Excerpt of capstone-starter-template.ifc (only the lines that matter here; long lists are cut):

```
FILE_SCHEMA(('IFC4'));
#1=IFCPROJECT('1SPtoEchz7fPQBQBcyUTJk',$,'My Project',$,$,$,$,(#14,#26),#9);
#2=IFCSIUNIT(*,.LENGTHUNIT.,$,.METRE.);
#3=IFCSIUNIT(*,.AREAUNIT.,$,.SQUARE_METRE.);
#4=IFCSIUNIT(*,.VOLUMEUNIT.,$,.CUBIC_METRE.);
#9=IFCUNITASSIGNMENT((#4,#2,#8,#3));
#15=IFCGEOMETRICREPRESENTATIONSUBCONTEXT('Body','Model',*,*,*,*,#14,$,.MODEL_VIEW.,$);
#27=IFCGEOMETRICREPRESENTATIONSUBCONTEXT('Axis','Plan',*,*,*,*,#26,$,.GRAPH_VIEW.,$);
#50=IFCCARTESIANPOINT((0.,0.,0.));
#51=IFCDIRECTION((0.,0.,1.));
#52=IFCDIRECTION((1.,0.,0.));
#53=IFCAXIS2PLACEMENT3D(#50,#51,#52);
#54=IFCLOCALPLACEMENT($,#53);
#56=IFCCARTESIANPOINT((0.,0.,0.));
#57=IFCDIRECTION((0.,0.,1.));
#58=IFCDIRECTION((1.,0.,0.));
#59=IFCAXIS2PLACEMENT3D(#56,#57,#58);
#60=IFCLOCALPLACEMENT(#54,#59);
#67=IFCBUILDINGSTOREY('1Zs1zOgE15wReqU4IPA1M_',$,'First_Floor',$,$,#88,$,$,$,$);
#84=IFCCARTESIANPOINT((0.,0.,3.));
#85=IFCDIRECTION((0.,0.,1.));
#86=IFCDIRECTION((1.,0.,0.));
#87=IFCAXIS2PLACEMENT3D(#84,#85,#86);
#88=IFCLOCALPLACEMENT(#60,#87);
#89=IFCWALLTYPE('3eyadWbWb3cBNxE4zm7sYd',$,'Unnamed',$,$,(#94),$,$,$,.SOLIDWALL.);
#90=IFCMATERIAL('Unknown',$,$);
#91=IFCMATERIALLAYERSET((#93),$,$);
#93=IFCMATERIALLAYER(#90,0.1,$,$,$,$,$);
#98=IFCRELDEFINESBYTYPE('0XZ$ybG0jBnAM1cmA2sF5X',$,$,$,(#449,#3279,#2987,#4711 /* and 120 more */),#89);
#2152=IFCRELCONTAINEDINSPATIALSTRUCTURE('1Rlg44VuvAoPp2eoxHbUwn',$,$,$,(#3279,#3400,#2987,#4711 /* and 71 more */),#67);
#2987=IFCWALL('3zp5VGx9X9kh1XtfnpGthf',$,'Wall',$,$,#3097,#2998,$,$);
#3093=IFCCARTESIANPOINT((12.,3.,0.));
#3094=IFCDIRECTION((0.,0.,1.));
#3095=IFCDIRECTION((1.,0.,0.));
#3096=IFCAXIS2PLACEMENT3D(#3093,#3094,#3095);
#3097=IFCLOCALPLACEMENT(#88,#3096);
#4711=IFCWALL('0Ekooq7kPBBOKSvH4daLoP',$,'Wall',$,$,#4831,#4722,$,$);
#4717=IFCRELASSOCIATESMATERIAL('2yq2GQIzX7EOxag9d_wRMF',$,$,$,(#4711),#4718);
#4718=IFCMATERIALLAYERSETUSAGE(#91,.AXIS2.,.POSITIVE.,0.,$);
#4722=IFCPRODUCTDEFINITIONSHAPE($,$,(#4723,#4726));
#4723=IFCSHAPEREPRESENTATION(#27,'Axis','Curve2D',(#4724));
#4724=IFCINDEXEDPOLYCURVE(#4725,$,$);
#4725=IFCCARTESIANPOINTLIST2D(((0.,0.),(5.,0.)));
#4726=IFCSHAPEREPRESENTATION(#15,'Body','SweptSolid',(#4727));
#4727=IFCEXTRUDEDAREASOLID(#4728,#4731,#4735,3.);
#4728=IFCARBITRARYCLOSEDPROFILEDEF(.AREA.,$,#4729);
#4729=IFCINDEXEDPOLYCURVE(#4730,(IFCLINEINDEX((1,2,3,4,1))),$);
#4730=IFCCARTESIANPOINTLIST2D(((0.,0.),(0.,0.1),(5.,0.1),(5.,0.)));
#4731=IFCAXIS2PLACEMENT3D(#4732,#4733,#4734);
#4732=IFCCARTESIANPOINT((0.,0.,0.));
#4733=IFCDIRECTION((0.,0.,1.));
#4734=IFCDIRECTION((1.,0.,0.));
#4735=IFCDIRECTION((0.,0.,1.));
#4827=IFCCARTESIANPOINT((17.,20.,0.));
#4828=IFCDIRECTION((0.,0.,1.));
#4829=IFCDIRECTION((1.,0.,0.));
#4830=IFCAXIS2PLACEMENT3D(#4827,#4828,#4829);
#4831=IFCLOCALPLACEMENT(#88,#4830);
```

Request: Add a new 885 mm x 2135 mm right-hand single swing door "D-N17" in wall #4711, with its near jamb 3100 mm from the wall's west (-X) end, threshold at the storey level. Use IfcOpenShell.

```python
import numpy as np
import ifcopenshell
import ifcopenshell.api.feature
import ifcopenshell.api.geometry
import ifcopenshell.api.root
import ifcopenshell.api.spatial
import ifcopenshell.geom
import ifcopenshell.util.element
import ifcopenshell.util.placement
import ifcopenshell.util.representation
import ifcopenshell.util.shape
import ifcopenshell.util.unit

model = ifcopenshell.open("capstone-starter-template.ifc")
unit_scale = ifcopenshell.util.unit.calculate_unit_scale(model)
settings = ifcopenshell.geom.settings()


def volume(element):
    """Net volume in cubic metres, openings subtracted."""
    shape = ifcopenshell.geom.create_shape(settings, element)
    return ifcopenshell.util.shape.get_volume(shape.geometry)


wall = model.by_guid("0Ekooq7kPBBOKSvH4daLoP")
storey = ifcopenshell.util.element.get_container(wall, ifc_class="IfcBuildingStorey")
context = ifcopenshell.util.representation.get_context(model, "Model", "Body", "MODEL_VIEW")
before = volume(wall)

width, height, from_end, sill = 0.885, 2.135, 3.1, 0.0  # metres

# The wall runs along its own X axis, and the end named is its -X end.
wall_shape = ifcopenshell.geom.create_shape(settings, wall)
x, y, z = ifcopenshell.util.shape.get_vertices(wall_shape.geometry).T
start = x.min() + from_end
face, thickness = float(y.min()), float(y.max() - y.min())
wall_matrix = ifcopenshell.util.placement.get_local_placement(wall.ObjectPlacement)
level = ifcopenshell.util.placement.get_local_placement(storey.ObjectPlacement)[2, 3]


def in_wall(x, y):
    """Placement at x, y metres in the wall's axes, at sill height."""
    matrix = wall_matrix.copy()
    matrix[:, 3] = wall_matrix @ np.array([x / unit_scale, y / unit_scale, 0.0, 1.0])
    matrix[2, 3] = level + sill / unit_scale
    return matrix


# Opening: a box that overshoots both wall faces by 50 mm.
opening = ifcopenshell.api.root.create_entity(model, ifc_class="IfcOpeningElement", predefined_type="OPENING")
box = ifcopenshell.api.geometry.add_wall_representation(
    model, context=context, length=width, height=height, thickness=thickness + 0.1
)
ifcopenshell.api.geometry.assign_representation(model, product=opening, representation=box)
ifcopenshell.api.geometry.edit_object_placement(model, product=opening, matrix=in_wall(start, face - 0.05), is_si=False)
ifcopenshell.api.feature.add_feature(model, feature=opening, element=wall)

door = ifcopenshell.api.root.create_entity(model, ifc_class="IfcDoor", name="D-N17", predefined_type="DOOR")
door.OverallWidth, door.OverallHeight = width / unit_scale, height / unit_scale
door.OperationType = "SINGLE_SWING_RIGHT"
body = ifcopenshell.api.geometry.add_door_representation(
    model,
    context=context,
    overall_width=door.OverallWidth,
    overall_height=door.OverallHeight,
    operation_type="SINGLE_SWING_RIGHT",
    lining_properties={"LiningDepth": thickness / unit_scale, "ThresholdDepth": thickness / unit_scale},
)
ifcopenshell.api.geometry.assign_representation(model, product=door, representation=body)
ifcopenshell.api.spatial.assign_container(model, products=[door], relating_structure=storey)
ifcopenshell.api.feature.add_filling(model, opening=opening, element=door)

# The lining spans the wall, so the door starts at the wall face.
ifcopenshell.api.geometry.edit_object_placement(model, product=door, matrix=in_wall(start, face), is_si=False)

after = volume(wall)

print(f"wall volume {before:.3f} -> {after:.3f} m3")

model.write("capstone-starter-template_updated.ifc")
```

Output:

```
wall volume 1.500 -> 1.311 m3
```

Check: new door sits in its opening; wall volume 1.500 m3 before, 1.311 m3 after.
